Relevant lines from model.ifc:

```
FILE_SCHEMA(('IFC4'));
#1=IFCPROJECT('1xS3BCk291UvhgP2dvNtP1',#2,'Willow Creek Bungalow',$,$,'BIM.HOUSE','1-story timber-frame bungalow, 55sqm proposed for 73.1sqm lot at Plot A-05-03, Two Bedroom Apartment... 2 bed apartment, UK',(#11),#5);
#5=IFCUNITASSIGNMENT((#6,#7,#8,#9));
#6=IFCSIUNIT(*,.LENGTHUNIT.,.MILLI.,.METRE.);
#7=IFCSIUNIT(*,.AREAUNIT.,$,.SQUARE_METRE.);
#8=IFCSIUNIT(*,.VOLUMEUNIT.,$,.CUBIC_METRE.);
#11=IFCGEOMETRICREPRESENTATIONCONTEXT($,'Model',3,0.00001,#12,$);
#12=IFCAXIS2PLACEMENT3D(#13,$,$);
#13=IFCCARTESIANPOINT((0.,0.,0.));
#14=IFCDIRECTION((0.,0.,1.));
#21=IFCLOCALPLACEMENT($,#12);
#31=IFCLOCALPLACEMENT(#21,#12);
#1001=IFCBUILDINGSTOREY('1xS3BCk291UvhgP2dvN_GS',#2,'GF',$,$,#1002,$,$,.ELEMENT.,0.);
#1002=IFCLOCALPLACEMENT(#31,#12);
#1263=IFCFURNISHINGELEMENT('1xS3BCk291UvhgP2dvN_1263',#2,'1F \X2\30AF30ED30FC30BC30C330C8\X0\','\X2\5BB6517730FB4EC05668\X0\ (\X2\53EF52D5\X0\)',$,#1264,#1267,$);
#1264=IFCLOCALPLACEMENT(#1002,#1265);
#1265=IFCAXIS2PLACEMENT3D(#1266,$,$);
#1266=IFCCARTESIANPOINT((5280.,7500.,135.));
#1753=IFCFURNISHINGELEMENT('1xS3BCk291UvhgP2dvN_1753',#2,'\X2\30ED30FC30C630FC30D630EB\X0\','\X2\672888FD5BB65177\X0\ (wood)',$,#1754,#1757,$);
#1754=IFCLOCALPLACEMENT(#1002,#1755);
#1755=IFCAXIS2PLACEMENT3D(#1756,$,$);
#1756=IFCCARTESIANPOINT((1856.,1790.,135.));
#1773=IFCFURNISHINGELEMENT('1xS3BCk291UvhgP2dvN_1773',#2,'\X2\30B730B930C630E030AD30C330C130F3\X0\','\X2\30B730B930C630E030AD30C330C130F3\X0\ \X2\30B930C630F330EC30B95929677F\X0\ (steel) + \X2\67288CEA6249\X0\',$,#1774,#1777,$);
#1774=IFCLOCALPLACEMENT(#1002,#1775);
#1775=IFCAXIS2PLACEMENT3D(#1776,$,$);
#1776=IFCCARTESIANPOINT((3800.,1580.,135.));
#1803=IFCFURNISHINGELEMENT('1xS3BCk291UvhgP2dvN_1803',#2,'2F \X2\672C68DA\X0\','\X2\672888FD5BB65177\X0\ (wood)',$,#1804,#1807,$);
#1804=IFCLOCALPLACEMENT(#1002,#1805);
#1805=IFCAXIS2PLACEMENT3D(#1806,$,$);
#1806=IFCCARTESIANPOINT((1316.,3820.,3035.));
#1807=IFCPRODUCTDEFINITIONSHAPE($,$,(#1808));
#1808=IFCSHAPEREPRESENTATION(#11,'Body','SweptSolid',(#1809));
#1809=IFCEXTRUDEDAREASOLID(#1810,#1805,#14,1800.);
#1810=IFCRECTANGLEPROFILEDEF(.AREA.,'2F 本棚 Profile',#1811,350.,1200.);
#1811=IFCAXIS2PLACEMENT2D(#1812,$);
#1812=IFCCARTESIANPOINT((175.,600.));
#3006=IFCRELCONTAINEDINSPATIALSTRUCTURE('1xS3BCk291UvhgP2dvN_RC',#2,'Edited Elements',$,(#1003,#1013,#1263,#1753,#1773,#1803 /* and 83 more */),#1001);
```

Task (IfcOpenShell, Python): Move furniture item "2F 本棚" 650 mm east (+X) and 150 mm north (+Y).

```python
import ifcopenshell
import ifcopenshell.api.geometry
import ifcopenshell.util.placement
import ifcopenshell.util.unit

model = ifcopenshell.open("model.ifc")
unit_scale = ifcopenshell.util.unit.calculate_unit_scale(model)

item = model.by_guid("1xS3BCk291UvhgP2dvN_1803")
matrix = ifcopenshell.util.placement.get_local_placement(item.ObjectPlacement)
matrix[0, 3] += 0.65 / unit_scale
matrix[1, 3] += 0.15 / unit_scale
ifcopenshell.api.geometry.edit_object_placement(model, product=item, matrix=matrix, is_si=False)

print(ifcopenshell.util.placement.get_local_placement(item.ObjectPlacement).round(3) + 0.0)

model.write("model_updated.ifc")
```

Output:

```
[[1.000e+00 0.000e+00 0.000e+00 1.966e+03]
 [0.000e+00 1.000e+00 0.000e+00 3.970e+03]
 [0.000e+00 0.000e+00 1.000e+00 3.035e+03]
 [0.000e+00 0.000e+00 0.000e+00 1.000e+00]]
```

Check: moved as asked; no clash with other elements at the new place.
